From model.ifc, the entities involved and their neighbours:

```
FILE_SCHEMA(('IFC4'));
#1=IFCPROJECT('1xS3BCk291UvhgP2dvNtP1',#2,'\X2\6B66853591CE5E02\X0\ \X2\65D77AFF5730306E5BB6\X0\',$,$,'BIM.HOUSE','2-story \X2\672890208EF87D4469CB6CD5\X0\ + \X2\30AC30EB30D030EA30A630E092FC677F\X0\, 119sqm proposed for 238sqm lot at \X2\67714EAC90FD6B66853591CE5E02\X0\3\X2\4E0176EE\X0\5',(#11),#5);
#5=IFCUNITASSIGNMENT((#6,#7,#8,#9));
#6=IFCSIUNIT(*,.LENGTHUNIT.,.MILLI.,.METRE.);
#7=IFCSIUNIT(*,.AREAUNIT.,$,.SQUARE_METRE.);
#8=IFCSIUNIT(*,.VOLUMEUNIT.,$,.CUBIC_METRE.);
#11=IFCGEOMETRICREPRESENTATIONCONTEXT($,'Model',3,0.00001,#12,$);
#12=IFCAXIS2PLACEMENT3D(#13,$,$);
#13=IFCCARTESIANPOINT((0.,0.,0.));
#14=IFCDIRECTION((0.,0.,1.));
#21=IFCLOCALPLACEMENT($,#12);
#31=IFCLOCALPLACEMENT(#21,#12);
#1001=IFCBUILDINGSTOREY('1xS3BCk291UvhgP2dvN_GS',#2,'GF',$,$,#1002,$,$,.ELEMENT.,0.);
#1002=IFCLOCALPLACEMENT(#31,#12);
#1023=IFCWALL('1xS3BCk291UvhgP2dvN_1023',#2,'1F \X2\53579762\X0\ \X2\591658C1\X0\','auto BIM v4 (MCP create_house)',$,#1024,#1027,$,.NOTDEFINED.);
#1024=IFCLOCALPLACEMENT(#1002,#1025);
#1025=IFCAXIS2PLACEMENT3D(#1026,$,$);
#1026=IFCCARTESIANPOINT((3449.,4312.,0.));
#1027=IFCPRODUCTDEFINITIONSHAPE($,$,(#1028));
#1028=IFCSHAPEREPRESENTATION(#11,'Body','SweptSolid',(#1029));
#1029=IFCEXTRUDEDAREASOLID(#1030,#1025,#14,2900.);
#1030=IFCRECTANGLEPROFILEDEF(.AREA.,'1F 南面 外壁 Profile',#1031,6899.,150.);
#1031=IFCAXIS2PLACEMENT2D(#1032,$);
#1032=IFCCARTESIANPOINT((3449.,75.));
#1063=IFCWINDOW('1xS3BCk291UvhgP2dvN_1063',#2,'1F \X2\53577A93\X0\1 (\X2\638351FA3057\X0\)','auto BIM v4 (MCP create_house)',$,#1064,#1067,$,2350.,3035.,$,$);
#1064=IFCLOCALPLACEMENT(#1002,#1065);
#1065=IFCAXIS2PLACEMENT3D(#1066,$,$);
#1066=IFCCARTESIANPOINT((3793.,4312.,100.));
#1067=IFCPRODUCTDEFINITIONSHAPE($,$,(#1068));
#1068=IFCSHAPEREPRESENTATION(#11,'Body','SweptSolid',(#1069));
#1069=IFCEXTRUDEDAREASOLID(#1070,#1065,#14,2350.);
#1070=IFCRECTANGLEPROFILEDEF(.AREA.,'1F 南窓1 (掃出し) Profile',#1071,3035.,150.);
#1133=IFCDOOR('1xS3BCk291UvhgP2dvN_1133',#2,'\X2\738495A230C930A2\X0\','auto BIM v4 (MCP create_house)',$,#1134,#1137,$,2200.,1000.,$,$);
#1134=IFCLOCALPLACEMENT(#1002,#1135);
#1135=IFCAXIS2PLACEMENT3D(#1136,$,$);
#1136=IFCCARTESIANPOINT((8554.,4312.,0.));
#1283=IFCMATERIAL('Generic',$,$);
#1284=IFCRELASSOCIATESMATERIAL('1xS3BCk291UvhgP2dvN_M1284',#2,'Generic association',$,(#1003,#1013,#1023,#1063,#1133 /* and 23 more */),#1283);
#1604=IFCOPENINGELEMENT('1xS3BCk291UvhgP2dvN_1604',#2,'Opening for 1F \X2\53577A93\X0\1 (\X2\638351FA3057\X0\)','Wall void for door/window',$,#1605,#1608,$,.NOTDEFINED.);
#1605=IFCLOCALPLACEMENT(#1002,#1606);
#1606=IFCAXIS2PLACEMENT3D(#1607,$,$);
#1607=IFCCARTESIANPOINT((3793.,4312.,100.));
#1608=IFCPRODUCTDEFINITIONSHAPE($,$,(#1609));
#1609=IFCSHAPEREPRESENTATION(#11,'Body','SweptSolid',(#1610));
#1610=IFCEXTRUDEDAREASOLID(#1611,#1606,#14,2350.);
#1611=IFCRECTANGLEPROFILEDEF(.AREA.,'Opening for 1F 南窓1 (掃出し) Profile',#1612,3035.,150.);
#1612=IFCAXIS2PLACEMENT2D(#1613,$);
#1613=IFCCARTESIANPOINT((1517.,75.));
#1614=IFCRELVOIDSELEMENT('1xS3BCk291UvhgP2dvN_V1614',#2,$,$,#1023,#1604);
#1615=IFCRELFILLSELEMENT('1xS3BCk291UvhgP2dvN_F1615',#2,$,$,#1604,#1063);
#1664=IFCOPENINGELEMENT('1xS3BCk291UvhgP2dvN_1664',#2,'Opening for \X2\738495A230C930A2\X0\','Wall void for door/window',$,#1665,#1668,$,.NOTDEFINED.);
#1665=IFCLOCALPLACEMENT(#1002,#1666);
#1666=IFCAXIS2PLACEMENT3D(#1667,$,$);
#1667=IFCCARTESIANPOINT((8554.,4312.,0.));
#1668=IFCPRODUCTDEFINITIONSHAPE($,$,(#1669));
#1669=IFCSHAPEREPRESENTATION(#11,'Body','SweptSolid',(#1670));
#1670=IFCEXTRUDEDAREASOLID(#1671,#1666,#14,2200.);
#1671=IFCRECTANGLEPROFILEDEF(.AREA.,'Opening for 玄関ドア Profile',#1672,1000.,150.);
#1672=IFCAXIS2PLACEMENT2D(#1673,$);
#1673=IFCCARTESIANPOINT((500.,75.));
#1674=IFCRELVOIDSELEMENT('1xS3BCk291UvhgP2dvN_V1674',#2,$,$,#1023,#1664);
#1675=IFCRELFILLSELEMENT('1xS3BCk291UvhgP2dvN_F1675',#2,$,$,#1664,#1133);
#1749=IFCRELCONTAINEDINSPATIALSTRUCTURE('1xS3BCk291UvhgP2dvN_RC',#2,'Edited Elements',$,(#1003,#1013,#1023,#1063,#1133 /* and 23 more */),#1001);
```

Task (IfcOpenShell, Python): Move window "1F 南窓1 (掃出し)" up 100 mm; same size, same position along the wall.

```python
import numpy as np
import ifcopenshell
import ifcopenshell.api.geometry
import ifcopenshell.util.placement
import ifcopenshell.util.unit

model = ifcopenshell.open("model.ifc")
unit_scale = ifcopenshell.util.unit.calculate_unit_scale(model)

window = model.by_guid("1xS3BCk291UvhgP2dvN_1063")
opening = window.FillsVoids[0].RelatingOpeningElement
dz = 100.0

shift = np.array([0.0, 0.0, dz])
# The window is not placed relative to its opening, so move both.
for product in (opening, window):
    matrix = ifcopenshell.util.placement.get_local_placement(product.ObjectPlacement)
    matrix[:3, 3] += shift
    ifcopenshell.api.geometry.edit_object_placement(model, product=product, matrix=matrix, is_si=False)

print(f"moved by {dz * unit_scale:+.3f} m")

model.write("model_rev.ifc")
```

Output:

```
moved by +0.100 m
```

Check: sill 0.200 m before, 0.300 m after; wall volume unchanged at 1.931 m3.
